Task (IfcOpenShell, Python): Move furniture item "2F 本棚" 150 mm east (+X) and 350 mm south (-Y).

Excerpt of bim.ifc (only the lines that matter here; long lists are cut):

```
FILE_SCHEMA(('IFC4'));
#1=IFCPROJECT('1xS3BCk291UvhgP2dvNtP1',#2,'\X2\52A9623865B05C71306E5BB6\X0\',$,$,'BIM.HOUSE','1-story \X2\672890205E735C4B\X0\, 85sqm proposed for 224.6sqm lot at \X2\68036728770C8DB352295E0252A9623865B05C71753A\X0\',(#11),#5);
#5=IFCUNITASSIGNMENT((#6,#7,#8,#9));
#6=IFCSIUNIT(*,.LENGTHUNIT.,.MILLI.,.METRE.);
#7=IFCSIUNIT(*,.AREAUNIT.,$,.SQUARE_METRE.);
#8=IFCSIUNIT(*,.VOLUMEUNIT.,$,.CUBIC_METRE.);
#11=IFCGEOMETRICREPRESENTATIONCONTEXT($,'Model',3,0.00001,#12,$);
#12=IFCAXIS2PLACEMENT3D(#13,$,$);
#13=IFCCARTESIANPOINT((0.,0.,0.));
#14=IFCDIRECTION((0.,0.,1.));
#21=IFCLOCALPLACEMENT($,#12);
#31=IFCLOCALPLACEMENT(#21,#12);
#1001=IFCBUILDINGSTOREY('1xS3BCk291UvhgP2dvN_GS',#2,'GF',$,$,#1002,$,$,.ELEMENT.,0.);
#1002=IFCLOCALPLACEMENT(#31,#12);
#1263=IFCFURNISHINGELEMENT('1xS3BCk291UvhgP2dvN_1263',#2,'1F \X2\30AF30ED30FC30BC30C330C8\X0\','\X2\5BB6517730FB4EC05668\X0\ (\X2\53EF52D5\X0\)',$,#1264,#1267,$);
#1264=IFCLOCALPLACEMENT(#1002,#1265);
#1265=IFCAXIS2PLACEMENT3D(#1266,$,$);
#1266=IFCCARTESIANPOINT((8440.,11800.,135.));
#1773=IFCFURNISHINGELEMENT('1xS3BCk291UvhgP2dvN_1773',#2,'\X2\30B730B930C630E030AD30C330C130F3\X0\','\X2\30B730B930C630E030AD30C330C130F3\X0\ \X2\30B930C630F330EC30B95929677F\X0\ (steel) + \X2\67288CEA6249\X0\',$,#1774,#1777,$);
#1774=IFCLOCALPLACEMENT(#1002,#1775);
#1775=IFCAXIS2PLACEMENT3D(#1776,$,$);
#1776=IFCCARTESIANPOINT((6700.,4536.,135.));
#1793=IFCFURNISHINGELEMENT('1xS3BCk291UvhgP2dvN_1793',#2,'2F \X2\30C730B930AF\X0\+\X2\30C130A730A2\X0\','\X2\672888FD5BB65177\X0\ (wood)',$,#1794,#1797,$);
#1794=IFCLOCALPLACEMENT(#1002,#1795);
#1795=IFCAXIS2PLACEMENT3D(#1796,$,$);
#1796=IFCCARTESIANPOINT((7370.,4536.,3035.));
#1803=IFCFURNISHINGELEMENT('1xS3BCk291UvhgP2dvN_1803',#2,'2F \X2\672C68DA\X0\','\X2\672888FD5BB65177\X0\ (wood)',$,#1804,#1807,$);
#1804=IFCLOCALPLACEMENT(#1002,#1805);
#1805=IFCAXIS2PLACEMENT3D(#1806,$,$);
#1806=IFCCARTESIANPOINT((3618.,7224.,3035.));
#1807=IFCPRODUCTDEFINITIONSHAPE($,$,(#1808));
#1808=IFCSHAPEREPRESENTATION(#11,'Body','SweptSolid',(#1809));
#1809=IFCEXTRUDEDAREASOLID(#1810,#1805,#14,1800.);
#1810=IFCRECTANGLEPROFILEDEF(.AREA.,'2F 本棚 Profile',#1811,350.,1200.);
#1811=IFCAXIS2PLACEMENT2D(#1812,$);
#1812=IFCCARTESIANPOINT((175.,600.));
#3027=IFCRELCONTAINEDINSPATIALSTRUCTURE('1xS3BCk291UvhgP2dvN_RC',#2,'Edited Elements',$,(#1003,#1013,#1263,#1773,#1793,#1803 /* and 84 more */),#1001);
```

```python
import ifcopenshell
import ifcopenshell.api.geometry
import ifcopenshell.util.placement
import ifcopenshell.util.unit

model = ifcopenshell.open("bim.ifc")
unit_scale = ifcopenshell.util.unit.calculate_unit_scale(model)

item = model.by_guid("1xS3BCk291UvhgP2dvN_1803")
matrix = ifcopenshell.util.placement.get_local_placement(item.ObjectPlacement)
matrix[0, 3] += 0.15 / unit_scale
matrix[1, 3] -= 0.35 / unit_scale
ifcopenshell.api.geometry.edit_object_placement(model, product=item, matrix=matrix, is_si=False)

print(ifcopenshell.util.placement.get_local_placement(item.ObjectPlacement).round(3) + 0.0)

model.write("bim-out.ifc")
```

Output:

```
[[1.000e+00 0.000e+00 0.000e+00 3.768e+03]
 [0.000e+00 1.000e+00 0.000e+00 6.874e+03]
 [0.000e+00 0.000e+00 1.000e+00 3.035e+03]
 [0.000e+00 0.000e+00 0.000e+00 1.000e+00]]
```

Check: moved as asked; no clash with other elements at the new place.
